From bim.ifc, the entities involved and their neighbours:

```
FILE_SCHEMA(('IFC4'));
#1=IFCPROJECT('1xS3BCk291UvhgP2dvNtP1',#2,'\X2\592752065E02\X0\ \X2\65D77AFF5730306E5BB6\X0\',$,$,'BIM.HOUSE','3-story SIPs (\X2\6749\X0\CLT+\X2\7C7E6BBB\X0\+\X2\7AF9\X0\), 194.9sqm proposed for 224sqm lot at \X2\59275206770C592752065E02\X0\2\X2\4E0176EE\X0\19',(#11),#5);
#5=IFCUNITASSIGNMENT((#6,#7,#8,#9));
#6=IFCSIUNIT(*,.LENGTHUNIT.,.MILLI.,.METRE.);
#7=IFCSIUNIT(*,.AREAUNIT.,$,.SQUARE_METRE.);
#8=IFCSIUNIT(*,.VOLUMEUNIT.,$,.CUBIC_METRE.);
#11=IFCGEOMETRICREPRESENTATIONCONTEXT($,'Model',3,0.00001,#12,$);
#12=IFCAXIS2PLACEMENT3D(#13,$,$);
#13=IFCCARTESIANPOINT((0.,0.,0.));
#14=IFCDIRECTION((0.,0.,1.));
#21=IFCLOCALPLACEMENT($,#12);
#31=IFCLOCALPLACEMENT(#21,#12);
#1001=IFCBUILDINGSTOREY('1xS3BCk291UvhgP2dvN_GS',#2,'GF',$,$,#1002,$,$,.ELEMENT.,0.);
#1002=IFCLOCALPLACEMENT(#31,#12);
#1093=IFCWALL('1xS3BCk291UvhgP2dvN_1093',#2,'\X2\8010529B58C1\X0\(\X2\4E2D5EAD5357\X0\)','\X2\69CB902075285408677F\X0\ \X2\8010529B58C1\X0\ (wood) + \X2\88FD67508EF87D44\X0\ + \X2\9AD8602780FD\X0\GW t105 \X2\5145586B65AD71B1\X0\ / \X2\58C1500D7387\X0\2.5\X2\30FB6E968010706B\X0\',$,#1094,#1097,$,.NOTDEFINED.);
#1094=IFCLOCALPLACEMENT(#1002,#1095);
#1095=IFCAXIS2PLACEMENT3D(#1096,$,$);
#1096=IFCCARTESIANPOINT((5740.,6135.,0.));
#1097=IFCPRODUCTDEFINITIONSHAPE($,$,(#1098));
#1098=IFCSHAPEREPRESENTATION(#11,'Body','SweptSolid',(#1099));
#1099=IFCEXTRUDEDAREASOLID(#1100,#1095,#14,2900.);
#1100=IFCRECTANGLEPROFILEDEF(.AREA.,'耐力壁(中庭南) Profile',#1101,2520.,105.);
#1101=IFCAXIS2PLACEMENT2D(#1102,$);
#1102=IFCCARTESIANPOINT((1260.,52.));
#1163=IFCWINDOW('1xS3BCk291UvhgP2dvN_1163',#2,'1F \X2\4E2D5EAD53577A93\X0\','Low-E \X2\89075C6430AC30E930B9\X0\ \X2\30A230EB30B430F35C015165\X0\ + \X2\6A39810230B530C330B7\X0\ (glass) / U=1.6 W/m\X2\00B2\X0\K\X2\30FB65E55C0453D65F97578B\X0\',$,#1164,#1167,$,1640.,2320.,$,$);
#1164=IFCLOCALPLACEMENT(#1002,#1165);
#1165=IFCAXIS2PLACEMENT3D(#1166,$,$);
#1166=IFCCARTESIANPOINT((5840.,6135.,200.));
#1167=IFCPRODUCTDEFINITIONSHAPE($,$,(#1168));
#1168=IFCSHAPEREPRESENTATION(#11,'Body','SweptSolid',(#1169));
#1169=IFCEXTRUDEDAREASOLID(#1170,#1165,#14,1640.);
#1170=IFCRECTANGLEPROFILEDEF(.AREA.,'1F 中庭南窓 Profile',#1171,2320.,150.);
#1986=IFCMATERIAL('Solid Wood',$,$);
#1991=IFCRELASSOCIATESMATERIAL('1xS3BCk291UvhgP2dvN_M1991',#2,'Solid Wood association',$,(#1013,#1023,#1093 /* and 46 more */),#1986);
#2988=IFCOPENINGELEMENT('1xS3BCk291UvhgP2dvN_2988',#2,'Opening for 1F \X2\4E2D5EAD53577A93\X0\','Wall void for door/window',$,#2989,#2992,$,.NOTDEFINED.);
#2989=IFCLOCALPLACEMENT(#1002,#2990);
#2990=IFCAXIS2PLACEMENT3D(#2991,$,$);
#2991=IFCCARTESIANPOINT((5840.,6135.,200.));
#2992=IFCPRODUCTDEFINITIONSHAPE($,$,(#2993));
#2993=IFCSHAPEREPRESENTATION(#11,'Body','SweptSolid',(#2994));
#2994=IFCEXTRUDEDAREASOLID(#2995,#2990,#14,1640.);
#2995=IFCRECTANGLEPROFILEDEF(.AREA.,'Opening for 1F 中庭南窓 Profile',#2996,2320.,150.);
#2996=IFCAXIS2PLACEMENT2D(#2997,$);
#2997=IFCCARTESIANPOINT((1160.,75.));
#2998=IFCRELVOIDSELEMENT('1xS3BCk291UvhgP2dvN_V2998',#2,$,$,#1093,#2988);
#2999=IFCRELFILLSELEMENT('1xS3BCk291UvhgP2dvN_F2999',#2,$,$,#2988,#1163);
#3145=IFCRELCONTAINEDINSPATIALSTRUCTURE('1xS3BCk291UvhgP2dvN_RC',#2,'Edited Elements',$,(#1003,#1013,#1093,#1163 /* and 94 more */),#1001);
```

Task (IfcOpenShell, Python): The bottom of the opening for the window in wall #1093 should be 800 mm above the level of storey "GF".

```python
import numpy as np
import ifcopenshell
import ifcopenshell.api.geometry
import ifcopenshell.geom
import ifcopenshell.util.element
import ifcopenshell.util.placement
import ifcopenshell.util.shape
import ifcopenshell.util.unit

model = ifcopenshell.open("bim.ifc")
unit_scale = ifcopenshell.util.unit.calculate_unit_scale(model)

window = model.by_id(1163)
opening = window.FillsVoids[0].RelatingOpeningElement
storey = ifcopenshell.util.element.get_container(window, ifc_class="IfcBuildingStorey")
level = ifcopenshell.util.placement.get_local_placement(storey.ObjectPlacement)[2, 3]

# The opening's origin need not be at the sill, so measure its lowest point.
shape = ifcopenshell.geom.create_shape(ifcopenshell.geom.settings(), opening)
bottom = ifcopenshell.util.shape.get_shape_bottom_elevation(shape, shape.geometry) / unit_scale
dz = level + 800.0 - bottom

shift = np.array([0.0, 0.0, dz])
# The window is not placed relative to its opening, so move both.
for product in (opening, window):
    matrix = ifcopenshell.util.placement.get_local_placement(product.ObjectPlacement)
    matrix[:3, 3] += shift
    ifcopenshell.api.geometry.edit_object_placement(model, product=product, matrix=matrix, is_si=False)

print(f"moved by {dz * unit_scale:+.3f} m")

model.write("bim_v2.ifc")
```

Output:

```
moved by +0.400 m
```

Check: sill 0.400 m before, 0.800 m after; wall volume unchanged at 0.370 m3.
